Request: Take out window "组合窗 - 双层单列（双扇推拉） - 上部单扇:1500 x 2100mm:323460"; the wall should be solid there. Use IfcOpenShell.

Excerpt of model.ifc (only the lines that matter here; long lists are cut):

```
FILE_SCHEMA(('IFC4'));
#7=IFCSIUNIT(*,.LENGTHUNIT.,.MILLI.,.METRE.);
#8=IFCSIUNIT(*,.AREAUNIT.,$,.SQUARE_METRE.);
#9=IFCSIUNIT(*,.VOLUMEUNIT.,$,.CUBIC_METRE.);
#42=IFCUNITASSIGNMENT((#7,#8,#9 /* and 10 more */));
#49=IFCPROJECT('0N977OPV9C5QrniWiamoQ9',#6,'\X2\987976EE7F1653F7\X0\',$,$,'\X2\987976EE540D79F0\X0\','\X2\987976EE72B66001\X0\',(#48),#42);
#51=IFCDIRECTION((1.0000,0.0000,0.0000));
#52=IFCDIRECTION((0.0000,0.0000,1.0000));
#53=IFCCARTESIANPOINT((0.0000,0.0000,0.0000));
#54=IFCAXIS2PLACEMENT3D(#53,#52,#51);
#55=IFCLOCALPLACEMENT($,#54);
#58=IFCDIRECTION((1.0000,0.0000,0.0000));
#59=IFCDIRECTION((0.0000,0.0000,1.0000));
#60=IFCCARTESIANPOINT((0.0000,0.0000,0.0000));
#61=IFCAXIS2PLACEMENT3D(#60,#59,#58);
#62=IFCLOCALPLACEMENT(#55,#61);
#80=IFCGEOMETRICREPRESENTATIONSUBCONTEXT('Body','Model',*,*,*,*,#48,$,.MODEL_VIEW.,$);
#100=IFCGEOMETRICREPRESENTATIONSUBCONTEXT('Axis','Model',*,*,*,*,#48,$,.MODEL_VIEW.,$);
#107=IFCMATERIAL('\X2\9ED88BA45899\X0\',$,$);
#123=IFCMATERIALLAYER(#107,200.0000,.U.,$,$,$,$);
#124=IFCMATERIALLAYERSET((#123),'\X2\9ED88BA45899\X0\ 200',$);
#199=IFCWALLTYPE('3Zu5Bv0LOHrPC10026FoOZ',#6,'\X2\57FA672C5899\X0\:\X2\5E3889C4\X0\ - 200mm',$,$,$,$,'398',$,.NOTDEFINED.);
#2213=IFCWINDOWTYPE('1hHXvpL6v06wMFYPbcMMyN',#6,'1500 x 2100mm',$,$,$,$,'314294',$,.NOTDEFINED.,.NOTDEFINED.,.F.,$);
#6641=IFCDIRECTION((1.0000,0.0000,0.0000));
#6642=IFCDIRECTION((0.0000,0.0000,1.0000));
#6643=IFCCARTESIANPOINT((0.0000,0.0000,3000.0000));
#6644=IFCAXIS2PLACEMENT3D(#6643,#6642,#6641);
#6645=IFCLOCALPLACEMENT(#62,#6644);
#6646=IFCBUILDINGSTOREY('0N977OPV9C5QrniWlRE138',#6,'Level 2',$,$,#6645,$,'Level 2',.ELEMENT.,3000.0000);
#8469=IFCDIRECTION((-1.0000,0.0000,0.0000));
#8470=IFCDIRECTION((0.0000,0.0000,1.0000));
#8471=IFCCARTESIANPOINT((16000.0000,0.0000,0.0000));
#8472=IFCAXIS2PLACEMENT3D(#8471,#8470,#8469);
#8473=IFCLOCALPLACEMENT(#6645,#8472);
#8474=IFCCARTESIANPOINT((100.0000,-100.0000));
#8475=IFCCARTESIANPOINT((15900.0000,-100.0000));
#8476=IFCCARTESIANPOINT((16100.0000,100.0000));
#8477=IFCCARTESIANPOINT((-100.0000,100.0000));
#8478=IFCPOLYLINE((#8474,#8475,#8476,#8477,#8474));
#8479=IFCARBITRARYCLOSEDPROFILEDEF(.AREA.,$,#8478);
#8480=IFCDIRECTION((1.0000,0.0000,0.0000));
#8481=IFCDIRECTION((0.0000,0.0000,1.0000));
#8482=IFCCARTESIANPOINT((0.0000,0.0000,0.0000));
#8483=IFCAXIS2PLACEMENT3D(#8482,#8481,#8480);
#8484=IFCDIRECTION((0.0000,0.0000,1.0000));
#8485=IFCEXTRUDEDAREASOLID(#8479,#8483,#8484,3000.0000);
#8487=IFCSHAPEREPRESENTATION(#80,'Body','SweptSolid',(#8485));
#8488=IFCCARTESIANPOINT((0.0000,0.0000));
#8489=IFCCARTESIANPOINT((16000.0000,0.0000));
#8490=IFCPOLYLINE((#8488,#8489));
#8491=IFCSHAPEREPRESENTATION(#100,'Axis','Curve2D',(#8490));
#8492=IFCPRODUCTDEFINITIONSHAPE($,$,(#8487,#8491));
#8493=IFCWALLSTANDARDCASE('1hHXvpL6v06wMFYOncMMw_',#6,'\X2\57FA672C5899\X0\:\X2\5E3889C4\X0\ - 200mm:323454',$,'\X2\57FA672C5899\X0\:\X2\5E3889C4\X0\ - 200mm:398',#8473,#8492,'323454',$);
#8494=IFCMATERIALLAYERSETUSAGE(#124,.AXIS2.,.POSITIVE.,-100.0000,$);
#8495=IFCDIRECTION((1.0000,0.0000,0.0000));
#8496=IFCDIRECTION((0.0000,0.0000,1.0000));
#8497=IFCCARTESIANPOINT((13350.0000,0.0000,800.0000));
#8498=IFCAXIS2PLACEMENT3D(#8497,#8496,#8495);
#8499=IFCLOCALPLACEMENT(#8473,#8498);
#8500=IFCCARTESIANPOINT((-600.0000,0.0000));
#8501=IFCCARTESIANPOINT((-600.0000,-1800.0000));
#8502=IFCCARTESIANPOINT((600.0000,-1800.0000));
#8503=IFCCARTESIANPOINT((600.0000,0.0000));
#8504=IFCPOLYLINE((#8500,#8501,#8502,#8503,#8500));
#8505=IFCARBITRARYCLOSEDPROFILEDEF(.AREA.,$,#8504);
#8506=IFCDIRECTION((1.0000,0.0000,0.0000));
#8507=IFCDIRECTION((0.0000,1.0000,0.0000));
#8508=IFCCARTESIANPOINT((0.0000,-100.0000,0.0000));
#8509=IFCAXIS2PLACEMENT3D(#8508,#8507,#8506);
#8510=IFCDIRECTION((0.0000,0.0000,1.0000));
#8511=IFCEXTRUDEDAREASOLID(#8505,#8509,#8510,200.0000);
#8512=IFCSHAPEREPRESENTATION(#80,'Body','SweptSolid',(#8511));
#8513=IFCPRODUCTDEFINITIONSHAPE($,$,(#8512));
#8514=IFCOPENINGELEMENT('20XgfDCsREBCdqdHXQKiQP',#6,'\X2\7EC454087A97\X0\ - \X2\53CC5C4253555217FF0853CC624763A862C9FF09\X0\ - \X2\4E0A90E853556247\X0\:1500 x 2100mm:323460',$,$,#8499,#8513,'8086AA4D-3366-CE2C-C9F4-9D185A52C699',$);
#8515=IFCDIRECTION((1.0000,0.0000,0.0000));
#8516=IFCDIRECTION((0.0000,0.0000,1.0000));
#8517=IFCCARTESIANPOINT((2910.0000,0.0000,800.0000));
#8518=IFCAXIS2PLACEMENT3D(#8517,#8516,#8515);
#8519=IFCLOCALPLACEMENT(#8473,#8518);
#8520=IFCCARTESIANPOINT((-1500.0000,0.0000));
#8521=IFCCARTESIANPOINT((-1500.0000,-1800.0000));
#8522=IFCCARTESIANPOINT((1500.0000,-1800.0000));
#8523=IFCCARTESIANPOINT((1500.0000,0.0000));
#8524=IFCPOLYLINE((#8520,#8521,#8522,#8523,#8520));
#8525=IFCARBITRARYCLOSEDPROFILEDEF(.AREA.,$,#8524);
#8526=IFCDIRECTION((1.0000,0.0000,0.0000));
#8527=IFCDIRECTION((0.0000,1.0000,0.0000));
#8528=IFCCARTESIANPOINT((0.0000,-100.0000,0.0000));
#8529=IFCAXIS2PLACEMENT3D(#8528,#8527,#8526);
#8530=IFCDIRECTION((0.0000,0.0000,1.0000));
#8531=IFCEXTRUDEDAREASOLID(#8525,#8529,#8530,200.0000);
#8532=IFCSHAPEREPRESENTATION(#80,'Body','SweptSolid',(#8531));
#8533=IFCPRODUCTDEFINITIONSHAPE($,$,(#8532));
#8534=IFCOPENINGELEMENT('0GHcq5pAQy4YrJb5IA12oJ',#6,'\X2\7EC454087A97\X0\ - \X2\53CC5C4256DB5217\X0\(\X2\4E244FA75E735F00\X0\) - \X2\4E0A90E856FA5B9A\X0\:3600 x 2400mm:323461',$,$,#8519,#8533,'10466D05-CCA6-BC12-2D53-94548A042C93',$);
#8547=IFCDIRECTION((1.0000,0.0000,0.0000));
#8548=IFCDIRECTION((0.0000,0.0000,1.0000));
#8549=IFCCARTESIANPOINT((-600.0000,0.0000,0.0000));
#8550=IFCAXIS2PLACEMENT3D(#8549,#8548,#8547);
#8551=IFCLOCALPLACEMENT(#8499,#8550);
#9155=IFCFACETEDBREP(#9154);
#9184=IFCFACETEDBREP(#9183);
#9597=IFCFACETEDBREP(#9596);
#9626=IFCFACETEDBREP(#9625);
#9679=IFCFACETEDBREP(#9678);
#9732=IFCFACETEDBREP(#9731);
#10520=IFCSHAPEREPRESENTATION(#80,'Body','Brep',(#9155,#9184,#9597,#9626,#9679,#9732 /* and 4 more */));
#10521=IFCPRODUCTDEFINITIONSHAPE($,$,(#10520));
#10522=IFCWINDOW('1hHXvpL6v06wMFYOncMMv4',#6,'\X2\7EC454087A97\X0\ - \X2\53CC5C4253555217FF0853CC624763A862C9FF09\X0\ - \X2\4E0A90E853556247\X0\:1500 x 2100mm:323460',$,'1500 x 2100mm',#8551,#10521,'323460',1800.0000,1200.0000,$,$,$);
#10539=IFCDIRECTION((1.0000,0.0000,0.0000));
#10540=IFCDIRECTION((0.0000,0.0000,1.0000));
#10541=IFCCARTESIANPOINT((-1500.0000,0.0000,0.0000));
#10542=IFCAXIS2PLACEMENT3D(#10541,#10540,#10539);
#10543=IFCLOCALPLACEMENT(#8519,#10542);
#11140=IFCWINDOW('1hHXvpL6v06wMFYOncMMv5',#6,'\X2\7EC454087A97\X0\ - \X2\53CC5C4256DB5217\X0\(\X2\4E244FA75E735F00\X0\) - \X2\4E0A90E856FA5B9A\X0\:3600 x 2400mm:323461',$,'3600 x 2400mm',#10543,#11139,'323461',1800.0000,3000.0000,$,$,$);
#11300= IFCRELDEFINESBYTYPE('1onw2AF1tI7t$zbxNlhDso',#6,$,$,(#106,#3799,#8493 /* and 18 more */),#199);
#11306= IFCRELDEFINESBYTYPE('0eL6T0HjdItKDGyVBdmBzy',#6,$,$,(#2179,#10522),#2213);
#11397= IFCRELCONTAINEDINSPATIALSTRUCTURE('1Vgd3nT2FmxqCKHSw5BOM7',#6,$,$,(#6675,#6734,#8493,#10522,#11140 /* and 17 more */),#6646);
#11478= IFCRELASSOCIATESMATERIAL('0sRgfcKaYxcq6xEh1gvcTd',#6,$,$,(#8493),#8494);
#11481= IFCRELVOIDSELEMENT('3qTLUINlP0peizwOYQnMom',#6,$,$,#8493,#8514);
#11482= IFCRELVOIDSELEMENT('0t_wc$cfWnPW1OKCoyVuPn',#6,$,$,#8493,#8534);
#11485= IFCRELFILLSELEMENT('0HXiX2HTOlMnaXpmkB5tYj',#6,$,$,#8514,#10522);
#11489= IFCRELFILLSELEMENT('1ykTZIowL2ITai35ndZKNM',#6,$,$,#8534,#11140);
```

```python
import ifcopenshell
import ifcopenshell.api.feature
import ifcopenshell.api.root
import ifcopenshell.geom
import ifcopenshell.util.shape

model = ifcopenshell.open("model.ifc")
settings = ifcopenshell.geom.settings()


def volume(element):
    """Net volume in cubic metres, openings subtracted."""
    shape = ifcopenshell.geom.create_shape(settings, element)
    return ifcopenshell.util.shape.get_volume(shape.geometry)


window = model.by_id(10522)
opening = window.FillsVoids[0].RelatingOpeningElement
wall = opening.VoidsElements[0].RelatingBuildingElement
before = volume(wall)

ifcopenshell.api.root.remove_product(model, product=window)
ifcopenshell.api.feature.remove_feature(model, feature=opening)

after = volume(wall)

print(f"wall volume {before:.3f} -> {after:.3f} m3")

model.write("model-out.ifc")
```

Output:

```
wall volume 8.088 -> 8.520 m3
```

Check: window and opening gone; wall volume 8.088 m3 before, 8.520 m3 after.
